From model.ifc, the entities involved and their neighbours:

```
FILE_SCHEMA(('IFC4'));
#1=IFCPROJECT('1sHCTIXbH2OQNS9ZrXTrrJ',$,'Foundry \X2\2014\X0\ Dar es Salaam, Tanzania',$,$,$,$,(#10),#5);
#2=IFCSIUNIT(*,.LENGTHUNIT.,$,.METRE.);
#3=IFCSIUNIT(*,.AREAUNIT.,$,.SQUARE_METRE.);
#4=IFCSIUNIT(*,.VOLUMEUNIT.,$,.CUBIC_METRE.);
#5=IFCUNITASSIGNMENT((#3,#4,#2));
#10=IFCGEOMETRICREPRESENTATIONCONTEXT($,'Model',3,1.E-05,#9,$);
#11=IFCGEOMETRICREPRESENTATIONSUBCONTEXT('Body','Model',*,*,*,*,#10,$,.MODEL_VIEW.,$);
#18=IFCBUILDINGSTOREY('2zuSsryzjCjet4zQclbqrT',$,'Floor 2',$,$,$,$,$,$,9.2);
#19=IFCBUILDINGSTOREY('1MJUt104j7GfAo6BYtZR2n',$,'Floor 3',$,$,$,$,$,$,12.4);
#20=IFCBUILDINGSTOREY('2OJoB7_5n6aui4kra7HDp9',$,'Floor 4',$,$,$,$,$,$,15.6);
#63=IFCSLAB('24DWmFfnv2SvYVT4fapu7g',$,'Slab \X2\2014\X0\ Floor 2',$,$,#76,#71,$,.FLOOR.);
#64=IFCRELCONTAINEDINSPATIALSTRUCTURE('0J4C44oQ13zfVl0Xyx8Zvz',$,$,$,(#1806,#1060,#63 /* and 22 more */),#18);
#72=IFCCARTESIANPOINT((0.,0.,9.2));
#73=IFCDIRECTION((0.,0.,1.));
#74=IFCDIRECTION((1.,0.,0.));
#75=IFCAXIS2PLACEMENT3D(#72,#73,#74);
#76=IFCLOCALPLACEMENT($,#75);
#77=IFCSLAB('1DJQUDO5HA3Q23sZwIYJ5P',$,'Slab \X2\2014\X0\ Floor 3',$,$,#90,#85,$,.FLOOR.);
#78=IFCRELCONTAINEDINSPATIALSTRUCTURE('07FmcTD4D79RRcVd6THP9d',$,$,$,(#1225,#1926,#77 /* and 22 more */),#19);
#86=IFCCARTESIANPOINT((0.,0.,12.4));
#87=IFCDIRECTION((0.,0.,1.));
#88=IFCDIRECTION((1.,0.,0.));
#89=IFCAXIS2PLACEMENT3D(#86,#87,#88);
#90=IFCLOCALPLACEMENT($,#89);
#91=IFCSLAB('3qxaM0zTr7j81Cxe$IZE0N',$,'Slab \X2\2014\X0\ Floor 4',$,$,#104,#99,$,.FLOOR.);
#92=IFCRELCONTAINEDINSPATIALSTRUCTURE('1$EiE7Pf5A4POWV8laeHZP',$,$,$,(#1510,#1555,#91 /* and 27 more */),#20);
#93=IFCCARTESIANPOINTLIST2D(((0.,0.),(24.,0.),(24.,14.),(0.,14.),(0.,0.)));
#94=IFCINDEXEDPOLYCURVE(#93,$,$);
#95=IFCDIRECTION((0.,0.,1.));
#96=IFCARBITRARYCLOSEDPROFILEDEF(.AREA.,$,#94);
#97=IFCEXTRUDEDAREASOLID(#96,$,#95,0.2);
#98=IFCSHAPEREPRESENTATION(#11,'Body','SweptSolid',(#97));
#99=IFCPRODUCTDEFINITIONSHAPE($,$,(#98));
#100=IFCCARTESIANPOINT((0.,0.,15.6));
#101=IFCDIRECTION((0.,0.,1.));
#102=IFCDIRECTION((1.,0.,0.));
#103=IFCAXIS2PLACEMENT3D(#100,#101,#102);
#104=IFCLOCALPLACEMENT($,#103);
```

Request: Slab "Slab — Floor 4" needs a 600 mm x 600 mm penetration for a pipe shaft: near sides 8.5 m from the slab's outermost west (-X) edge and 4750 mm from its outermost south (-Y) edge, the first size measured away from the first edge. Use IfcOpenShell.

```python
import numpy as np
import ifcopenshell
import ifcopenshell.api.feature
import ifcopenshell.api.geometry
import ifcopenshell.api.root
import ifcopenshell.geom
import ifcopenshell.util.placement
import ifcopenshell.util.representation
import ifcopenshell.util.shape
import ifcopenshell.util.unit

model = ifcopenshell.open("model.ifc")
unit_scale = ifcopenshell.util.unit.calculate_unit_scale(model)
settings = ifcopenshell.geom.settings()


def volume(element):
    """Net volume in cubic metres, openings subtracted."""
    shape = ifcopenshell.geom.create_shape(settings, element)
    return ifcopenshell.util.shape.get_volume(shape.geometry)


slab = model.by_guid("3qxaM0zTr7j81Cxe$IZE0N")
before = volume(slab)

# Extent in the slab's own axes, in metres. The edges named are its -X and -Y sides.
slab_shape = ifcopenshell.geom.create_shape(settings, slab)
vertices = ifcopenshell.util.shape.get_vertices(slab_shape.geometry)
x_min, y_min, bottom = vertices.min(axis=0)
top = vertices[:, 2].max()

opening = ifcopenshell.api.root.create_entity(model, ifc_class="IfcOpeningElement", name="Pipe shaft opening", predefined_type="OPENING")
context = ifcopenshell.util.representation.get_context(model, "Model", "Body", "MODEL_VIEW")
width, depth = 0.6, 0.6
outline = [(0.0, 0.0), (width, 0.0), (width, depth), (0.0, depth), (0.0, 0.0)]
# Overshoot both faces by 50 mm so the cut is clean.
shape = ifcopenshell.api.geometry.add_slab_representation(
    model, context=context, depth=top - bottom + 0.1, polyline=outline
)
ifcopenshell.api.geometry.assign_representation(model, product=opening, representation=shape)

matrix = ifcopenshell.util.placement.get_local_placement(slab.ObjectPlacement)
matrix[:, 3] = matrix @ np.append(np.array([x_min + 8.5, y_min + 4.75, bottom - 0.05]) / unit_scale, 1.0)
ifcopenshell.api.geometry.edit_object_placement(model, product=opening, matrix=matrix, is_si=False)
ifcopenshell.api.feature.add_feature(model, feature=opening, element=slab)

after = volume(slab)

print(f"slab volume {before:.3f} -> {after:.3f} m3")

model.write("model_v2.ifc")
```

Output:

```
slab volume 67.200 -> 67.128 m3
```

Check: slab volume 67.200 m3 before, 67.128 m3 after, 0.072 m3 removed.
